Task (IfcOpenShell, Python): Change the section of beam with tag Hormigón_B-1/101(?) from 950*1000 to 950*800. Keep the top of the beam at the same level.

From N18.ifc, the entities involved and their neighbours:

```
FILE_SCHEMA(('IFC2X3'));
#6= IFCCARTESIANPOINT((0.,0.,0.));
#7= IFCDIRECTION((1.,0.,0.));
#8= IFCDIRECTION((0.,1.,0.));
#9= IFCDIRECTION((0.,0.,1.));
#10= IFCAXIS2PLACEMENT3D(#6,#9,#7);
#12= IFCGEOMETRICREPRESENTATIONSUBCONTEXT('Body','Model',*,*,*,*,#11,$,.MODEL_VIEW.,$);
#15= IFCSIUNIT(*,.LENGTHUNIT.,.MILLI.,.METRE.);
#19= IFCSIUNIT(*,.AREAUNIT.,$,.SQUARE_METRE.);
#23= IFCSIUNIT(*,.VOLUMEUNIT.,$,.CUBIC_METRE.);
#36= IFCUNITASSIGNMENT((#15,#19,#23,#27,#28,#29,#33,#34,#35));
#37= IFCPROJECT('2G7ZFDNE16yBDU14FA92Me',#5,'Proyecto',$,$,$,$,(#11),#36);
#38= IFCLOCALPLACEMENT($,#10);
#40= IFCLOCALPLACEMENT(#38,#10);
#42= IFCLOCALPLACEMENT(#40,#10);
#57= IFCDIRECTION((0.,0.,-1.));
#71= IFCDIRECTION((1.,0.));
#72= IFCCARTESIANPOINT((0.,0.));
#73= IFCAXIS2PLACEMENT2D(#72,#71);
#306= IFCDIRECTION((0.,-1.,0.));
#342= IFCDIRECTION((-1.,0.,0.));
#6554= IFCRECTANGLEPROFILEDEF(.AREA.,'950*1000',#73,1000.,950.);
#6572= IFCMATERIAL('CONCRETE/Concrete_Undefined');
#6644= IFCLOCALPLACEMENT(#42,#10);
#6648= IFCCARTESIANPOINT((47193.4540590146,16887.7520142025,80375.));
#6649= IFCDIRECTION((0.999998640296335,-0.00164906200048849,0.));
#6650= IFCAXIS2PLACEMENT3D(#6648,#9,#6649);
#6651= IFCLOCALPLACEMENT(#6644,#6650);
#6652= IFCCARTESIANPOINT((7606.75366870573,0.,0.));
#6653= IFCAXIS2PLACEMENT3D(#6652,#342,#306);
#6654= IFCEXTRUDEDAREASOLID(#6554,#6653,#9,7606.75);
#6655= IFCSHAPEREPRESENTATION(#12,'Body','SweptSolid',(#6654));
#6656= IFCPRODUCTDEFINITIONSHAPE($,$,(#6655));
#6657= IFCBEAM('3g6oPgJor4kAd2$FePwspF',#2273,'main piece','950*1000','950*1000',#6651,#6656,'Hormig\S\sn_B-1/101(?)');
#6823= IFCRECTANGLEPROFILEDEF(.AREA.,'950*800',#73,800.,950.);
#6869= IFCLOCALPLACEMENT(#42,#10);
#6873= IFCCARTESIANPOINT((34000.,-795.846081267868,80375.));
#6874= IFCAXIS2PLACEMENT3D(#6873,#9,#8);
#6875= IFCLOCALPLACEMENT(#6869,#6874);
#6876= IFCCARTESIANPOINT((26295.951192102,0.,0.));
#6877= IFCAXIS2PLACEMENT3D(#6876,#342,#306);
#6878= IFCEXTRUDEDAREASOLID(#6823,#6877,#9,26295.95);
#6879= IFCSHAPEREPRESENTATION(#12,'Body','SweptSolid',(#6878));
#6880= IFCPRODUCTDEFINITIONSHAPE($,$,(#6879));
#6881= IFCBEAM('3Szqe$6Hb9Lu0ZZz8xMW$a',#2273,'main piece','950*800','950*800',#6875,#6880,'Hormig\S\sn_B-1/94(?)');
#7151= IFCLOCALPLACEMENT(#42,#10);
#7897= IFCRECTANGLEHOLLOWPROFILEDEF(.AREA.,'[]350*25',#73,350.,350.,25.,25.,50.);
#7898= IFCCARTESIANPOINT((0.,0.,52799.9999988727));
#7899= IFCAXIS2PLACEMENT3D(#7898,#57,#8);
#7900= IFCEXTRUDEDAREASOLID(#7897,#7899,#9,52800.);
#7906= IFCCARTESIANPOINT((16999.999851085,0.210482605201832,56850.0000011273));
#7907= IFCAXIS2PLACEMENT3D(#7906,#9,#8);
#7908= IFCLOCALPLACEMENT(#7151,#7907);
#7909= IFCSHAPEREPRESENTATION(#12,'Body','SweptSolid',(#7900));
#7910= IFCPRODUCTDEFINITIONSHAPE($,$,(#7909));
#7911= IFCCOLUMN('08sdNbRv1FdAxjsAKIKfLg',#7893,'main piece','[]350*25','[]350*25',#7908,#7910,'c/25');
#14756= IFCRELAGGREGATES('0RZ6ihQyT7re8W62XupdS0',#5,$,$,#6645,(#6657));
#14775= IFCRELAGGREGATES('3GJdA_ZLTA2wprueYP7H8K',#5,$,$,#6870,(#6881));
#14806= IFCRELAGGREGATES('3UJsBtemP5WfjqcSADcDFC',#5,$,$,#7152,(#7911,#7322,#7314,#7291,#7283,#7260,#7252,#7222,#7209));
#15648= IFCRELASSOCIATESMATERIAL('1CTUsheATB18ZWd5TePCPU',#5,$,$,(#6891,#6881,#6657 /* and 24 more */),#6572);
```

```python
import ifcopenshell
import ifcopenshell.util.element
import ifcopenshell.util.representation

model = ifcopenshell.open("N18.ifc")

member = model.by_guid("3g6oPgJor4kAd2$FePwspF")
source = next(p for p in model.by_type("IfcRectangleProfileDef") if p.ProfileName == "950*800")

body = ifcopenshell.util.representation.get_representation(member, "Model", "Body")
solid = body.Items[0]
old_profile = solid.SweptArea

# Copy the section's sizes but keep this member's own profile position.
profile = ifcopenshell.util.element.copy(model, source)
# Profiles are centred, so shift by half the change in depth to hold the top.
shift = (old_profile.YDim - profile.YDim) / 2
x, y = old_profile.Position.Location.Coordinates
up = (0.0, 1.0)  # upwards, in the solid's own plane
location = model.createIfcCartesianPoint((x + up[0] * shift, y + up[1] * shift))
profile.Position = model.createIfcAxis2Placement2D(location, old_profile.Position.RefDirection)
solid.SweptArea = profile
if not model.get_total_inverses(old_profile):
    ifcopenshell.util.element.remove_deep2(model, old_profile)
member.Description = member.Description.replace("950*1000", "950*800")
member.ObjectType = member.ObjectType.replace("950*1000", "950*800")

print(solid.SweptArea)

model.write("N18_edited.ifc")
```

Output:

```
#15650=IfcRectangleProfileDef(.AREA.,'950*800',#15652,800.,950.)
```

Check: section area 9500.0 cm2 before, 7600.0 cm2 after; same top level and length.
